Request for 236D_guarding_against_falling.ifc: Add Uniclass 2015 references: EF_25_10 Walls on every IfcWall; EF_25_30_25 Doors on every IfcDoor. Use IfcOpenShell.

First a look at what the model holds.

```python
import ifcopenshell

model = ifcopenshell.open("236D_guarding_against_falling.ifc")
print(model.schema)
print("classifications:", [c.Name for c in model.by_type("IfcClassification")])
for ifc_class in ("IfcDoor", "IfcRoof", "IfcStair", "IfcWall", "IfcWindow"):
    print(ifc_class, len(model.by_type(ifc_class)))
```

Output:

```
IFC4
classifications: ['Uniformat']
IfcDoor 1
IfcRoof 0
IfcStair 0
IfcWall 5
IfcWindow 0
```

```python
import ifcopenshell
import ifcopenshell.api.classification

model = ifcopenshell.open("236D_guarding_against_falling.ifc")

system = ifcopenshell.api.classification.add_classification(model, classification="Uniclass 2015")

codes = {
    "IfcWall": ("EF_25_10", "Walls"),
    "IfcDoor": ("EF_25_30_25", "Doors"),
}
for ifc_class, (code, name) in codes.items():
    products = model.by_type(ifc_class)
    ifcopenshell.api.classification.add_reference(
        model, products=products, classification=system, identification=code, name=name
    )
    print(code, len(products))

model.write("236D_guarding_against_falling_rev.ifc")
```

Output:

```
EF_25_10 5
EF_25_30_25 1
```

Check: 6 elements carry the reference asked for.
